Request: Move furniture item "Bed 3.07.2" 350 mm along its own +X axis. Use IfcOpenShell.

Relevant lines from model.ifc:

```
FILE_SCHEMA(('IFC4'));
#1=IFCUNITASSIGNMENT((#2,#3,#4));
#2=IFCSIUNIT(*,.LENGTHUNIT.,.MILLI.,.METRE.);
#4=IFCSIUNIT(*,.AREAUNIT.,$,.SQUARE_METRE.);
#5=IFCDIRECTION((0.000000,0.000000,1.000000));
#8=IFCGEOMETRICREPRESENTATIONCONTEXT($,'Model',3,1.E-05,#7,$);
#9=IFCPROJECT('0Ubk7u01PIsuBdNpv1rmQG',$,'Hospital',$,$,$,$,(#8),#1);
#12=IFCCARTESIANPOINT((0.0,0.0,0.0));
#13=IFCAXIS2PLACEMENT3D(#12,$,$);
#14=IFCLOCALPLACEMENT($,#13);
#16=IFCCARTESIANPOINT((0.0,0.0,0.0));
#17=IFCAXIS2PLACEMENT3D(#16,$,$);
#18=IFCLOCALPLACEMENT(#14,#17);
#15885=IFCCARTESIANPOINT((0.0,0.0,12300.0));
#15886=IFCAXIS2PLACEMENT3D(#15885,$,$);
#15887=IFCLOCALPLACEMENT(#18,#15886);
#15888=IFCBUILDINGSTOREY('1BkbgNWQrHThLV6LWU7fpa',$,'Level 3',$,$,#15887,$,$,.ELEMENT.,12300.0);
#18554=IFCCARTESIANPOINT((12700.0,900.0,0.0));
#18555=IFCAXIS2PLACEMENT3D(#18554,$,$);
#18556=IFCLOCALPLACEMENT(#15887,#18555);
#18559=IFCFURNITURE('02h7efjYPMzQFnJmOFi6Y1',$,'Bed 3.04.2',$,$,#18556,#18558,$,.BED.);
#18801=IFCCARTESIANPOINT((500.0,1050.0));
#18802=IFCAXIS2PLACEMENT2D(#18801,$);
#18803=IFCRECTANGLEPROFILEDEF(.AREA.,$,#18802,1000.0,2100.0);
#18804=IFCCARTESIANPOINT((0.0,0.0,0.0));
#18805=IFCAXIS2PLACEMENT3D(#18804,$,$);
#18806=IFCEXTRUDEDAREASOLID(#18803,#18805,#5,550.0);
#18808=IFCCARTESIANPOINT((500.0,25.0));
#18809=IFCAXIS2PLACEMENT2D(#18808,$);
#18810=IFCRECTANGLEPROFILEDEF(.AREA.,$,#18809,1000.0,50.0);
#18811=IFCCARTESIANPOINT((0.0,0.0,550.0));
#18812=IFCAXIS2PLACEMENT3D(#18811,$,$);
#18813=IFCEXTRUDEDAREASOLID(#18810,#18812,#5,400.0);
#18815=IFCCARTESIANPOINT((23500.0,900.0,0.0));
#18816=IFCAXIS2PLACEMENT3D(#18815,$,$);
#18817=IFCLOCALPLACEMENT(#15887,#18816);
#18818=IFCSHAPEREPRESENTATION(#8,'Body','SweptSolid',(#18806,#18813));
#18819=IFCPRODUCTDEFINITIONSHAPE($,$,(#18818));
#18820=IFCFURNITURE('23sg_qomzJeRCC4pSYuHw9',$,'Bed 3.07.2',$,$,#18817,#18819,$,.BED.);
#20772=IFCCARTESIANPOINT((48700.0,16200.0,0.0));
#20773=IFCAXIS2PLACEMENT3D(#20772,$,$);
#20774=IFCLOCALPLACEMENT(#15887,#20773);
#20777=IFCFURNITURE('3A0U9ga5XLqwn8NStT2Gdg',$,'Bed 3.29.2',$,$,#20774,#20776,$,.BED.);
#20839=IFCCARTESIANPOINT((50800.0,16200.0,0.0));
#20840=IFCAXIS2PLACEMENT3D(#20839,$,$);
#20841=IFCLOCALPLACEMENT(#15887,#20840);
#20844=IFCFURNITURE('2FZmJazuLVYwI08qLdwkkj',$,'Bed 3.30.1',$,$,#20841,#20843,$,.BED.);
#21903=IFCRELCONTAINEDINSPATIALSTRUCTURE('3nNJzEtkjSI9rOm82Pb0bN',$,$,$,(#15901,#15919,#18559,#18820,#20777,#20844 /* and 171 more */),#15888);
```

```python
import ifcopenshell
import ifcopenshell.api.geometry
import ifcopenshell.util.placement
import ifcopenshell.util.unit

model = ifcopenshell.open("model.ifc")
unit_scale = ifcopenshell.util.unit.calculate_unit_scale(model)

item = model.by_id(18820)
matrix = ifcopenshell.util.placement.get_local_placement(item.ObjectPlacement)
matrix[:3, 3] += matrix[:3, 0] * 0.35 / unit_scale
ifcopenshell.api.geometry.edit_object_placement(model, product=item, matrix=matrix, is_si=False)

print(ifcopenshell.util.placement.get_local_placement(item.ObjectPlacement).round(3) + 0.0)

model.write("model_edited.ifc")
```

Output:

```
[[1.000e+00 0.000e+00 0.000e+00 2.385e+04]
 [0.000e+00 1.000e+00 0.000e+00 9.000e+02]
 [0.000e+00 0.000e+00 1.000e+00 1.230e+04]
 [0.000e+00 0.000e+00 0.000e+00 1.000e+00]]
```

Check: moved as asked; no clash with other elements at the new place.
